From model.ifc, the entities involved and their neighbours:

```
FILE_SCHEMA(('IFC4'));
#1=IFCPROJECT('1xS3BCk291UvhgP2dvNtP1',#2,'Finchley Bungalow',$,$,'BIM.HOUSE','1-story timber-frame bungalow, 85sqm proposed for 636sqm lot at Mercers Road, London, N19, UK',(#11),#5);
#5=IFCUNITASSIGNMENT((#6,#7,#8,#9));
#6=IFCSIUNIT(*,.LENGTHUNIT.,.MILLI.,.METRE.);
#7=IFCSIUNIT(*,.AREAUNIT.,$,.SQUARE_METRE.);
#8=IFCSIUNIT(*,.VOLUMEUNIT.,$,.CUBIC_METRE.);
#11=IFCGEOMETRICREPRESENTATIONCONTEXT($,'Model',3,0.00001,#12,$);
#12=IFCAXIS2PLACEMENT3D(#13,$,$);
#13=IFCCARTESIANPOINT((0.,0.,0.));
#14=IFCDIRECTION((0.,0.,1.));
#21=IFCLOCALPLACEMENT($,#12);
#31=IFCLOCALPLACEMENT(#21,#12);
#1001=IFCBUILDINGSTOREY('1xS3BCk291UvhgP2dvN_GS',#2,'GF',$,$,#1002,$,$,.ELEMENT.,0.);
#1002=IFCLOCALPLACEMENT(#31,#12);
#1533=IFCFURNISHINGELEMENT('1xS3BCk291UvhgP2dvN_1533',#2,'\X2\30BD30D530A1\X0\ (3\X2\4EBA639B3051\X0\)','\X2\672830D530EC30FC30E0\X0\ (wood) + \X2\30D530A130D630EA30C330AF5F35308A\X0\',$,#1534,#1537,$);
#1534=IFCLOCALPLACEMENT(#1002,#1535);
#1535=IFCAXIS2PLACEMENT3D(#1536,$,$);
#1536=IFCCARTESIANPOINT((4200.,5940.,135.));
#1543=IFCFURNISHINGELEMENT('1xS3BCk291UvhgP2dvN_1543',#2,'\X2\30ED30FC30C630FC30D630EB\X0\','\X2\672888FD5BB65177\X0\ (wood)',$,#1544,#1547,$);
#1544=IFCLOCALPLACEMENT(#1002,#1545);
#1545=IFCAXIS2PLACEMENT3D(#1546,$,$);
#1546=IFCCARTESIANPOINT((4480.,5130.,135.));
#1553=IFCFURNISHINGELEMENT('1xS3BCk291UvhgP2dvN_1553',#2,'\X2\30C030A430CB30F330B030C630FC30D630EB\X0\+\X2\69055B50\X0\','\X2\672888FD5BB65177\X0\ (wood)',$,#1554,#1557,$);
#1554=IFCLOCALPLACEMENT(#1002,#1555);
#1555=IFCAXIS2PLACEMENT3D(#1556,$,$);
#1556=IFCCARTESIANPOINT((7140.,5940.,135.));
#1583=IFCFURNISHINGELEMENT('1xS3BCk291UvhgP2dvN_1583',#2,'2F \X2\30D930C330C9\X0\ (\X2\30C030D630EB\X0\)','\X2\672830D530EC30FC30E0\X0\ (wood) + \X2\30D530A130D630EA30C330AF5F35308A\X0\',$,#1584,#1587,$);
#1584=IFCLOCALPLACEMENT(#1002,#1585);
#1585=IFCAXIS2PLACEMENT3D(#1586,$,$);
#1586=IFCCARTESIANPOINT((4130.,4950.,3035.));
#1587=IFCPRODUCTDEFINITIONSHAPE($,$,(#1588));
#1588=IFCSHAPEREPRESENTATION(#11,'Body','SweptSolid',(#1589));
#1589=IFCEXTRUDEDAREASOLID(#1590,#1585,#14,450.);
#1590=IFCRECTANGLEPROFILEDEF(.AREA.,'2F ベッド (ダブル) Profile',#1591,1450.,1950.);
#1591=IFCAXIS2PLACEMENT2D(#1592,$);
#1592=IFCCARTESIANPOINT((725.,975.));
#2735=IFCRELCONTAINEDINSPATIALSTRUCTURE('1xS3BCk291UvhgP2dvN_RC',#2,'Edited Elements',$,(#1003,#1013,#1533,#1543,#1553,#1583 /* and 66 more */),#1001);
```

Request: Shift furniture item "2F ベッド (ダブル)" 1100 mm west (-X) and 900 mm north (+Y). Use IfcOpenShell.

```python
import ifcopenshell
import ifcopenshell.api.geometry
import ifcopenshell.util.placement

model = ifcopenshell.open("model.ifc")

item = model.by_guid("1xS3BCk291UvhgP2dvN_1583")
matrix = ifcopenshell.util.placement.get_local_placement(item.ObjectPlacement)
matrix[0, 3] -= 1100.0
matrix[1, 3] += 900.0
ifcopenshell.api.geometry.edit_object_placement(model, product=item, matrix=matrix, is_si=False)

print(ifcopenshell.util.placement.get_local_placement(item.ObjectPlacement).round(3) + 0.0)

model.write("model_updated.ifc")
```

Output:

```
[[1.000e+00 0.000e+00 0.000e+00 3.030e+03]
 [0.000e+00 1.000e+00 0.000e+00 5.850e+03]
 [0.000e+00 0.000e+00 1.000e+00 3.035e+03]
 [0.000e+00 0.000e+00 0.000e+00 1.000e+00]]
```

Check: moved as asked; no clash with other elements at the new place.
